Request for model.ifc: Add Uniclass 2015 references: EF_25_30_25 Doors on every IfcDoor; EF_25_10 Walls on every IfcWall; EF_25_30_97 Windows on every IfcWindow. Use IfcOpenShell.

First a look at what the model holds.

```python
import ifcopenshell

model = ifcopenshell.open("model.ifc")
print(model.schema)
print("classifications:", [c.Name for c in model.by_type("IfcClassification")])
for ifc_class in ("IfcDoor", "IfcRoof", "IfcStair", "IfcWall", "IfcWindow"):
    print(ifc_class, len(model.by_type(ifc_class)))
```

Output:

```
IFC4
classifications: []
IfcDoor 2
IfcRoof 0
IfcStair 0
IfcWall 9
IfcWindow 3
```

```python
import ifcopenshell
import ifcopenshell.api.classification

model = ifcopenshell.open("model.ifc")

system = ifcopenshell.api.classification.add_classification(model, classification="Uniclass 2015")

codes = {
    "IfcDoor": ("EF_25_30_25", "Doors"),
    "IfcWall": ("EF_25_10", "Walls"),
    "IfcWindow": ("EF_25_30_97", "Windows"),
}
for ifc_class, (code, name) in codes.items():
    products = model.by_type(ifc_class)
    ifcopenshell.api.classification.add_reference(
        model, products=products, classification=system, identification=code, name=name
    )
    print(code, len(products))

model.write("model_rev.ifc")
```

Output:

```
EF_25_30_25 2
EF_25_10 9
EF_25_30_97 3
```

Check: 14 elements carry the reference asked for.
